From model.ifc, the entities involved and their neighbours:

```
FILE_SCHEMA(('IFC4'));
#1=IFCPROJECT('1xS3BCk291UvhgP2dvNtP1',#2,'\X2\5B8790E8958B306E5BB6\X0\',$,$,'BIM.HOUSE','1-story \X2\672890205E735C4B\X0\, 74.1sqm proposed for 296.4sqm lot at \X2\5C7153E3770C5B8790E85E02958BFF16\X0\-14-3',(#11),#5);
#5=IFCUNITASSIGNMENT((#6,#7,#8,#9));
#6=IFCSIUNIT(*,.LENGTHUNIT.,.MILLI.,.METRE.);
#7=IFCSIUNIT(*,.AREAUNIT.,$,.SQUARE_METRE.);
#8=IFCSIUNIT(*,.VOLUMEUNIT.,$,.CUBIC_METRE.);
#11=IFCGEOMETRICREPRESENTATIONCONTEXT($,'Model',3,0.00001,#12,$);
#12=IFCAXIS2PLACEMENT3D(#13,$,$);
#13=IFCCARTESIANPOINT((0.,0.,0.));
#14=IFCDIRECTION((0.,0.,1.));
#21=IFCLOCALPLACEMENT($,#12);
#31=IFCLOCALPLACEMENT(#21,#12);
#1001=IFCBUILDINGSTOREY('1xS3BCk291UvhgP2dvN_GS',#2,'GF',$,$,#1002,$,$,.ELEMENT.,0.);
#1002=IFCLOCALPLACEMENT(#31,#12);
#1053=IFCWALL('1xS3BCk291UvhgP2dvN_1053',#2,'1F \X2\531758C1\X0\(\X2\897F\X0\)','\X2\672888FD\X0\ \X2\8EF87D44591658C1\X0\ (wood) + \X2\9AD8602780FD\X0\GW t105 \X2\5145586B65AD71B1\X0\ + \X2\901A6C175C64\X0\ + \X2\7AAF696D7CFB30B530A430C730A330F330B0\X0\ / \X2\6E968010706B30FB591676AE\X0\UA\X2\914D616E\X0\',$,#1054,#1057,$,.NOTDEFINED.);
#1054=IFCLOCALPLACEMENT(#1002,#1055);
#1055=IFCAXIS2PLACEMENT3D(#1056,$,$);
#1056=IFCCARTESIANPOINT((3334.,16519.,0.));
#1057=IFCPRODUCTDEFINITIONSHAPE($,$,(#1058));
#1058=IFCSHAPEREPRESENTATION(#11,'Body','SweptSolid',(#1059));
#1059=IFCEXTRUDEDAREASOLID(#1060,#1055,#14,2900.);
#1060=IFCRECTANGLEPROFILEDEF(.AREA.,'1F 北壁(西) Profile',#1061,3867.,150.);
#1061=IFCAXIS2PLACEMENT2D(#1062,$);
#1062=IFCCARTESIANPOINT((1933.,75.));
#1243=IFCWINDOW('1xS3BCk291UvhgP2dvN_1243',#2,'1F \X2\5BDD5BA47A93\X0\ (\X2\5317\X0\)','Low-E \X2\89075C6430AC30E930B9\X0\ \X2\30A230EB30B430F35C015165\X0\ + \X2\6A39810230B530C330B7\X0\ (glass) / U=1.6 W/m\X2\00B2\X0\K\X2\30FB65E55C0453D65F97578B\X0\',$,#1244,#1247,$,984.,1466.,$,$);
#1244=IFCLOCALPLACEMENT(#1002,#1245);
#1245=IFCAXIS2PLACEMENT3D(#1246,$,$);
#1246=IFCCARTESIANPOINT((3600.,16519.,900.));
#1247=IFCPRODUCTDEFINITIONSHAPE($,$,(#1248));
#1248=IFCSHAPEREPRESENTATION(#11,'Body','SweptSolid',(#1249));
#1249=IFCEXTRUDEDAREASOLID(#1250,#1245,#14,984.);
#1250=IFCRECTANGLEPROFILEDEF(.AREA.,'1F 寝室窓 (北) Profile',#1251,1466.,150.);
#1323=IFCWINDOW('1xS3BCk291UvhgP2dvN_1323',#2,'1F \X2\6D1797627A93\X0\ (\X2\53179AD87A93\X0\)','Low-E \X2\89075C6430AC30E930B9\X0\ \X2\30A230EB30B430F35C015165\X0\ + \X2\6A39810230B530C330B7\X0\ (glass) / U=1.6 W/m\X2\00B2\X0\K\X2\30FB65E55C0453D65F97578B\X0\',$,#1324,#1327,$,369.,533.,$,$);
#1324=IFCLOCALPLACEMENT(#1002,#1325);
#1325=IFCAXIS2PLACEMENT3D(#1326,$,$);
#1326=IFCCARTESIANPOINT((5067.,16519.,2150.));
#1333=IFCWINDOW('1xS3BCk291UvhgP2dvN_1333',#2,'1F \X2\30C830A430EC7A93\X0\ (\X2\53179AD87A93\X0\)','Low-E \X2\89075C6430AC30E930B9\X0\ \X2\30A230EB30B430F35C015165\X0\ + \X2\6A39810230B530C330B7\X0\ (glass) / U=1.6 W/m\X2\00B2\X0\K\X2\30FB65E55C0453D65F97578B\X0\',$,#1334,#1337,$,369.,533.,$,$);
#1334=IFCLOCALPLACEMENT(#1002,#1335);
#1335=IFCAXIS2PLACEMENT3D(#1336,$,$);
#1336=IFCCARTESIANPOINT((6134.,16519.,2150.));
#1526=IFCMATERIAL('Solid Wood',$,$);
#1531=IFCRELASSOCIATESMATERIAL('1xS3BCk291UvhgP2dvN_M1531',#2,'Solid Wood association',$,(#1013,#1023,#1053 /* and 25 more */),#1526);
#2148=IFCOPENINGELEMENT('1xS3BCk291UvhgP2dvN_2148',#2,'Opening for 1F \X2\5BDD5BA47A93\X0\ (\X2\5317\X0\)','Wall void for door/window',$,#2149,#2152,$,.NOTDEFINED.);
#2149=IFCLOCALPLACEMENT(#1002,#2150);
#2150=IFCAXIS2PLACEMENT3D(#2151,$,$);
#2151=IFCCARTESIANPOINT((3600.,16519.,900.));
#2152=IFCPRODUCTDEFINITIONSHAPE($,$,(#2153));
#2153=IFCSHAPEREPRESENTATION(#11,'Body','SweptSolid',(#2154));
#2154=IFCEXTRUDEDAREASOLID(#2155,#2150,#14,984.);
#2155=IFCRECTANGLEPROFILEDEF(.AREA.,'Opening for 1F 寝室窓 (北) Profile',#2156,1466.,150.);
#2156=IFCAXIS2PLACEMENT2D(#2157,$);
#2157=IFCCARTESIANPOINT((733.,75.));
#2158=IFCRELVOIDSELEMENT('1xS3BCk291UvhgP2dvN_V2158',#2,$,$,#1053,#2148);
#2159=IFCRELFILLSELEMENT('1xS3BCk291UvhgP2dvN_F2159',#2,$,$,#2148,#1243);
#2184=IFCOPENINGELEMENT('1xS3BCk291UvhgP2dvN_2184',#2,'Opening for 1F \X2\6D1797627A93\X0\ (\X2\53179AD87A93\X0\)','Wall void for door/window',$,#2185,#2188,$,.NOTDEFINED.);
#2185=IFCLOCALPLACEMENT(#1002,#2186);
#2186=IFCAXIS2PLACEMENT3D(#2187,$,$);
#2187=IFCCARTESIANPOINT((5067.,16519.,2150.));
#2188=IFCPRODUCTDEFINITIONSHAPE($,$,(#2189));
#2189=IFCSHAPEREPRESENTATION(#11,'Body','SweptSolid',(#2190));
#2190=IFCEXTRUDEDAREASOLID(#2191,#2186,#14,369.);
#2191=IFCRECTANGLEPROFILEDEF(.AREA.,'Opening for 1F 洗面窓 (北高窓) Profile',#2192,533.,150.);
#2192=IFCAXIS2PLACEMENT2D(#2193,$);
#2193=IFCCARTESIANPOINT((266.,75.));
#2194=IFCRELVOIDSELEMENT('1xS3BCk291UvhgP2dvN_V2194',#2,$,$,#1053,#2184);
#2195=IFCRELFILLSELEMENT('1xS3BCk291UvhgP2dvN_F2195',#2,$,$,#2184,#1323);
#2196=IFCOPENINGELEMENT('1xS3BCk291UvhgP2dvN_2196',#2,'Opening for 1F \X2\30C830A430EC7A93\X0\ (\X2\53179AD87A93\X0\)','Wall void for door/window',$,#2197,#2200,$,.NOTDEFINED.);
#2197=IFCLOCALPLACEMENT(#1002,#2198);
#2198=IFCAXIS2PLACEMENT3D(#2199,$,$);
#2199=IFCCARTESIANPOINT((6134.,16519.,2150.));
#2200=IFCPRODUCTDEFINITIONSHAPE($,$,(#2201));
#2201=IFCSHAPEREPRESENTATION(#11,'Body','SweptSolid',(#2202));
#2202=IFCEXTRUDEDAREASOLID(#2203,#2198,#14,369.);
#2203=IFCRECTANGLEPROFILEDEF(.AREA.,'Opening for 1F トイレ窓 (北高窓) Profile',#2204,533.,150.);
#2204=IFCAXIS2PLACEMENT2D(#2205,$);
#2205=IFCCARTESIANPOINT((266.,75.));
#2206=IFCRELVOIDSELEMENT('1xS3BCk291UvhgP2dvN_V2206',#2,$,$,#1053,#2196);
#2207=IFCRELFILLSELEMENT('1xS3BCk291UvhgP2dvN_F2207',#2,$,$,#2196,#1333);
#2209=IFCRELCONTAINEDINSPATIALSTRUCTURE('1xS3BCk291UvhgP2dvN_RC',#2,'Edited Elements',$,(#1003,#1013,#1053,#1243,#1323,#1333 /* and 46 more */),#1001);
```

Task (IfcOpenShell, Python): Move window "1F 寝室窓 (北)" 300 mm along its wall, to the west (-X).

```python
import ifcopenshell
import ifcopenshell.api.geometry
import ifcopenshell.util.placement
import ifcopenshell.util.unit

model = ifcopenshell.open("model.ifc")
unit_scale = ifcopenshell.util.unit.calculate_unit_scale(model)

window = model.by_id(1243)
opening = window.FillsVoids[0].RelatingOpeningElement
wall = opening.VoidsElements[0].RelatingBuildingElement

wall_matrix = ifcopenshell.util.placement.get_local_placement(wall.ObjectPlacement)
shift = wall_matrix[:3, 0] * -0.3 / unit_scale
before = ifcopenshell.util.placement.get_local_placement(window.ObjectPlacement)[:3, 3].copy()

# The window is not placed relative to its opening, so move both.
for product in (opening, window):
    matrix = ifcopenshell.util.placement.get_local_placement(product.ObjectPlacement)
    matrix[:3, 3] += shift
    ifcopenshell.api.geometry.edit_object_placement(model, product=product, matrix=matrix, is_si=False)

after = ifcopenshell.util.placement.get_local_placement(window.ObjectPlacement)[:3, 3]
print("window moved by", (after - before).round(3) + 0.0)

model.write("model_edited.ifc")
```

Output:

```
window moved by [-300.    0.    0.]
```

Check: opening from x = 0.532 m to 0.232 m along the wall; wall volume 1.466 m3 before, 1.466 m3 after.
